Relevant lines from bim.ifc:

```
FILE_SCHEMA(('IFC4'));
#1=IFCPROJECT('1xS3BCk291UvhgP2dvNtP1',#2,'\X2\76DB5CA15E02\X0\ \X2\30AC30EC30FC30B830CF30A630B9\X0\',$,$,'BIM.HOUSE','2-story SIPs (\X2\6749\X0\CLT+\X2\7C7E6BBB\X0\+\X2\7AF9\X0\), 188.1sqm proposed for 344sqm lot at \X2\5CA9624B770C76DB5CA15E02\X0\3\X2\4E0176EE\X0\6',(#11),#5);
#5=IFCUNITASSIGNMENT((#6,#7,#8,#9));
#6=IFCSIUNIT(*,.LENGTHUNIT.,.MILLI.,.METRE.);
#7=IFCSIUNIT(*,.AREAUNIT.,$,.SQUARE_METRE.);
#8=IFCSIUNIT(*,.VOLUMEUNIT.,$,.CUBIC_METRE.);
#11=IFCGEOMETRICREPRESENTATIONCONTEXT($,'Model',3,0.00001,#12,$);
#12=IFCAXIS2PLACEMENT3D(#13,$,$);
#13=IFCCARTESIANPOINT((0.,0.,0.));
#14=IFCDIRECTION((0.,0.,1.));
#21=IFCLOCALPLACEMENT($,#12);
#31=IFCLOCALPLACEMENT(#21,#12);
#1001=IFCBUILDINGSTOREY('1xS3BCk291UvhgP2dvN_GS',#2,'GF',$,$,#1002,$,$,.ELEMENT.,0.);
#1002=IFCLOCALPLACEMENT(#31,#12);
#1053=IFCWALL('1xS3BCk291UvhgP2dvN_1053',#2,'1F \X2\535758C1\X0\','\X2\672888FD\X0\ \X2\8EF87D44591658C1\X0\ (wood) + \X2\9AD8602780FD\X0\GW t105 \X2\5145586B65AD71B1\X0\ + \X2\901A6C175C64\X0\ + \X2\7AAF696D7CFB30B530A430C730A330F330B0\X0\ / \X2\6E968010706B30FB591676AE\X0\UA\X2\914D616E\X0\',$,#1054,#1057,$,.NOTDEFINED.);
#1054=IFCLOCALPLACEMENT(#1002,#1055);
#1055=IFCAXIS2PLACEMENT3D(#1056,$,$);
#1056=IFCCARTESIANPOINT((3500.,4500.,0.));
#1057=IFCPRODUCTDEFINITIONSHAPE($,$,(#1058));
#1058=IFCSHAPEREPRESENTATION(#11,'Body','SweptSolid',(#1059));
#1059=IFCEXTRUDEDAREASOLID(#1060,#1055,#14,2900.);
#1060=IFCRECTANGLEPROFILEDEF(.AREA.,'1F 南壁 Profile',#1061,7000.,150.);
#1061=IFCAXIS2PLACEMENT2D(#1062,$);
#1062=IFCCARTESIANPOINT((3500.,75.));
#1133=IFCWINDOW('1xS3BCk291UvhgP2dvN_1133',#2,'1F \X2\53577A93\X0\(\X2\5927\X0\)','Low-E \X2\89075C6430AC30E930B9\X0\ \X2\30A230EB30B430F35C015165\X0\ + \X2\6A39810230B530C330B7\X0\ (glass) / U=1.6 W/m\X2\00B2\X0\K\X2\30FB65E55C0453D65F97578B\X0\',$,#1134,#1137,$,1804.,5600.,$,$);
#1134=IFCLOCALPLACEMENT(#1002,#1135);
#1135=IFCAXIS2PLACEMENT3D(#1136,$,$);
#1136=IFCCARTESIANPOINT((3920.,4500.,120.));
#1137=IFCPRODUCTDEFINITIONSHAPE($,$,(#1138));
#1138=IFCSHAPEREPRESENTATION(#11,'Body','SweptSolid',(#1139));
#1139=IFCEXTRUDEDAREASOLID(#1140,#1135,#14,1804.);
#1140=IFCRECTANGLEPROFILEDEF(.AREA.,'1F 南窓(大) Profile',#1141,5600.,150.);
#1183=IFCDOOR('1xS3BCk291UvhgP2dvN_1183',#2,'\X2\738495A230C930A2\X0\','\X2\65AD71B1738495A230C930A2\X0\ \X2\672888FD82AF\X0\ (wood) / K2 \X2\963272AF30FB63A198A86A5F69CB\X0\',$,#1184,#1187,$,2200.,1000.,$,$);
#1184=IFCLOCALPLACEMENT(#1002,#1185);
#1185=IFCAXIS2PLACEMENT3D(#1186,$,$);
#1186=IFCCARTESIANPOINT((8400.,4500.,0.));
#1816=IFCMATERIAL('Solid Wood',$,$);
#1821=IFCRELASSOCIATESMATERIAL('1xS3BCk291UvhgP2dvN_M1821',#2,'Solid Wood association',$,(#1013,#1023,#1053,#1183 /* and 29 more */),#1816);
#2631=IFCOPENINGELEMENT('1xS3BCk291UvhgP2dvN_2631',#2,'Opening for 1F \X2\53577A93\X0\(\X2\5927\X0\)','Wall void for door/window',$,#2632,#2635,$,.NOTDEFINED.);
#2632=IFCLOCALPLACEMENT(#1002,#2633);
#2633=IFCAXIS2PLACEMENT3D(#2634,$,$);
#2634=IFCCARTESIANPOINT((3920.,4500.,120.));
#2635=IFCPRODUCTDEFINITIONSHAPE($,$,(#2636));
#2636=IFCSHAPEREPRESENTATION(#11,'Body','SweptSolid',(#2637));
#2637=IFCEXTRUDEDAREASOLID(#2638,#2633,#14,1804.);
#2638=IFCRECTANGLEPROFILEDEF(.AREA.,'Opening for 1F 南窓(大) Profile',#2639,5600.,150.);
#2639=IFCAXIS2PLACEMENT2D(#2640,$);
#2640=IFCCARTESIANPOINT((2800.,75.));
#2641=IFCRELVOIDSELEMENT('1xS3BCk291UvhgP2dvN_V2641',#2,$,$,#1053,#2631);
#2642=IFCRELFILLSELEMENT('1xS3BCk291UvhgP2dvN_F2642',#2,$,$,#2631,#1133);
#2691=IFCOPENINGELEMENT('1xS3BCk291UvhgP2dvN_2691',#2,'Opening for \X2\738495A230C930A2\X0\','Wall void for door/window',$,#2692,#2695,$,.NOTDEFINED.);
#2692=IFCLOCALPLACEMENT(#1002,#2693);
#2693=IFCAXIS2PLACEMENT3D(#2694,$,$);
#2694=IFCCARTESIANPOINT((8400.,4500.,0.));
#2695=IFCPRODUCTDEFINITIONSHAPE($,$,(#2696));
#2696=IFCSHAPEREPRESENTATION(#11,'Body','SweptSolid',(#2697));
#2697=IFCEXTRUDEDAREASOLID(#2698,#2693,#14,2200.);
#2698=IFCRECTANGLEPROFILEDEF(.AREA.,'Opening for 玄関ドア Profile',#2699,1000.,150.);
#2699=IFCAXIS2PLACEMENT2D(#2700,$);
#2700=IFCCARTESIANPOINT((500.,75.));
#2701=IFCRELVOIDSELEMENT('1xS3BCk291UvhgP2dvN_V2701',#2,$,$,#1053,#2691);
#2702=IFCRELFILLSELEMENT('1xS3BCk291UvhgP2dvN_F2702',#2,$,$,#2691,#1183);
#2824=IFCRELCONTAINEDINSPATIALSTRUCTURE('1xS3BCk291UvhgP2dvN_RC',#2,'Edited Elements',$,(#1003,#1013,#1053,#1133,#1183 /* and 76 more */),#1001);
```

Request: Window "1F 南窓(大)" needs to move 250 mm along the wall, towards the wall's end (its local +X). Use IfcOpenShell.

```python
import ifcopenshell
import ifcopenshell.api.geometry
import ifcopenshell.util.placement
import ifcopenshell.util.unit

model = ifcopenshell.open("bim.ifc")
unit_scale = ifcopenshell.util.unit.calculate_unit_scale(model)

window = model.by_guid("1xS3BCk291UvhgP2dvN_1133")
opening = window.FillsVoids[0].RelatingOpeningElement
wall = opening.VoidsElements[0].RelatingBuildingElement

wall_matrix = ifcopenshell.util.placement.get_local_placement(wall.ObjectPlacement)
shift = wall_matrix[:3, 0] * 0.25 / unit_scale
before = ifcopenshell.util.placement.get_local_placement(window.ObjectPlacement)[:3, 3].copy()

# The window is not placed relative to its opening, so move both.
for product in (opening, window):
    matrix = ifcopenshell.util.placement.get_local_placement(product.ObjectPlacement)
    matrix[:3, 3] += shift
    ifcopenshell.api.geometry.edit_object_placement(model, product=product, matrix=matrix, is_si=False)

after = ifcopenshell.util.placement.get_local_placement(window.ObjectPlacement)[:3, 3]
print("window moved by", (after - before).round(3) + 0.0)

model.write("bim_updated.ifc")
```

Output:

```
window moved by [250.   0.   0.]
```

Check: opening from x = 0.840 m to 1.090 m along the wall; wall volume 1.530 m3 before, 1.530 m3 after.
